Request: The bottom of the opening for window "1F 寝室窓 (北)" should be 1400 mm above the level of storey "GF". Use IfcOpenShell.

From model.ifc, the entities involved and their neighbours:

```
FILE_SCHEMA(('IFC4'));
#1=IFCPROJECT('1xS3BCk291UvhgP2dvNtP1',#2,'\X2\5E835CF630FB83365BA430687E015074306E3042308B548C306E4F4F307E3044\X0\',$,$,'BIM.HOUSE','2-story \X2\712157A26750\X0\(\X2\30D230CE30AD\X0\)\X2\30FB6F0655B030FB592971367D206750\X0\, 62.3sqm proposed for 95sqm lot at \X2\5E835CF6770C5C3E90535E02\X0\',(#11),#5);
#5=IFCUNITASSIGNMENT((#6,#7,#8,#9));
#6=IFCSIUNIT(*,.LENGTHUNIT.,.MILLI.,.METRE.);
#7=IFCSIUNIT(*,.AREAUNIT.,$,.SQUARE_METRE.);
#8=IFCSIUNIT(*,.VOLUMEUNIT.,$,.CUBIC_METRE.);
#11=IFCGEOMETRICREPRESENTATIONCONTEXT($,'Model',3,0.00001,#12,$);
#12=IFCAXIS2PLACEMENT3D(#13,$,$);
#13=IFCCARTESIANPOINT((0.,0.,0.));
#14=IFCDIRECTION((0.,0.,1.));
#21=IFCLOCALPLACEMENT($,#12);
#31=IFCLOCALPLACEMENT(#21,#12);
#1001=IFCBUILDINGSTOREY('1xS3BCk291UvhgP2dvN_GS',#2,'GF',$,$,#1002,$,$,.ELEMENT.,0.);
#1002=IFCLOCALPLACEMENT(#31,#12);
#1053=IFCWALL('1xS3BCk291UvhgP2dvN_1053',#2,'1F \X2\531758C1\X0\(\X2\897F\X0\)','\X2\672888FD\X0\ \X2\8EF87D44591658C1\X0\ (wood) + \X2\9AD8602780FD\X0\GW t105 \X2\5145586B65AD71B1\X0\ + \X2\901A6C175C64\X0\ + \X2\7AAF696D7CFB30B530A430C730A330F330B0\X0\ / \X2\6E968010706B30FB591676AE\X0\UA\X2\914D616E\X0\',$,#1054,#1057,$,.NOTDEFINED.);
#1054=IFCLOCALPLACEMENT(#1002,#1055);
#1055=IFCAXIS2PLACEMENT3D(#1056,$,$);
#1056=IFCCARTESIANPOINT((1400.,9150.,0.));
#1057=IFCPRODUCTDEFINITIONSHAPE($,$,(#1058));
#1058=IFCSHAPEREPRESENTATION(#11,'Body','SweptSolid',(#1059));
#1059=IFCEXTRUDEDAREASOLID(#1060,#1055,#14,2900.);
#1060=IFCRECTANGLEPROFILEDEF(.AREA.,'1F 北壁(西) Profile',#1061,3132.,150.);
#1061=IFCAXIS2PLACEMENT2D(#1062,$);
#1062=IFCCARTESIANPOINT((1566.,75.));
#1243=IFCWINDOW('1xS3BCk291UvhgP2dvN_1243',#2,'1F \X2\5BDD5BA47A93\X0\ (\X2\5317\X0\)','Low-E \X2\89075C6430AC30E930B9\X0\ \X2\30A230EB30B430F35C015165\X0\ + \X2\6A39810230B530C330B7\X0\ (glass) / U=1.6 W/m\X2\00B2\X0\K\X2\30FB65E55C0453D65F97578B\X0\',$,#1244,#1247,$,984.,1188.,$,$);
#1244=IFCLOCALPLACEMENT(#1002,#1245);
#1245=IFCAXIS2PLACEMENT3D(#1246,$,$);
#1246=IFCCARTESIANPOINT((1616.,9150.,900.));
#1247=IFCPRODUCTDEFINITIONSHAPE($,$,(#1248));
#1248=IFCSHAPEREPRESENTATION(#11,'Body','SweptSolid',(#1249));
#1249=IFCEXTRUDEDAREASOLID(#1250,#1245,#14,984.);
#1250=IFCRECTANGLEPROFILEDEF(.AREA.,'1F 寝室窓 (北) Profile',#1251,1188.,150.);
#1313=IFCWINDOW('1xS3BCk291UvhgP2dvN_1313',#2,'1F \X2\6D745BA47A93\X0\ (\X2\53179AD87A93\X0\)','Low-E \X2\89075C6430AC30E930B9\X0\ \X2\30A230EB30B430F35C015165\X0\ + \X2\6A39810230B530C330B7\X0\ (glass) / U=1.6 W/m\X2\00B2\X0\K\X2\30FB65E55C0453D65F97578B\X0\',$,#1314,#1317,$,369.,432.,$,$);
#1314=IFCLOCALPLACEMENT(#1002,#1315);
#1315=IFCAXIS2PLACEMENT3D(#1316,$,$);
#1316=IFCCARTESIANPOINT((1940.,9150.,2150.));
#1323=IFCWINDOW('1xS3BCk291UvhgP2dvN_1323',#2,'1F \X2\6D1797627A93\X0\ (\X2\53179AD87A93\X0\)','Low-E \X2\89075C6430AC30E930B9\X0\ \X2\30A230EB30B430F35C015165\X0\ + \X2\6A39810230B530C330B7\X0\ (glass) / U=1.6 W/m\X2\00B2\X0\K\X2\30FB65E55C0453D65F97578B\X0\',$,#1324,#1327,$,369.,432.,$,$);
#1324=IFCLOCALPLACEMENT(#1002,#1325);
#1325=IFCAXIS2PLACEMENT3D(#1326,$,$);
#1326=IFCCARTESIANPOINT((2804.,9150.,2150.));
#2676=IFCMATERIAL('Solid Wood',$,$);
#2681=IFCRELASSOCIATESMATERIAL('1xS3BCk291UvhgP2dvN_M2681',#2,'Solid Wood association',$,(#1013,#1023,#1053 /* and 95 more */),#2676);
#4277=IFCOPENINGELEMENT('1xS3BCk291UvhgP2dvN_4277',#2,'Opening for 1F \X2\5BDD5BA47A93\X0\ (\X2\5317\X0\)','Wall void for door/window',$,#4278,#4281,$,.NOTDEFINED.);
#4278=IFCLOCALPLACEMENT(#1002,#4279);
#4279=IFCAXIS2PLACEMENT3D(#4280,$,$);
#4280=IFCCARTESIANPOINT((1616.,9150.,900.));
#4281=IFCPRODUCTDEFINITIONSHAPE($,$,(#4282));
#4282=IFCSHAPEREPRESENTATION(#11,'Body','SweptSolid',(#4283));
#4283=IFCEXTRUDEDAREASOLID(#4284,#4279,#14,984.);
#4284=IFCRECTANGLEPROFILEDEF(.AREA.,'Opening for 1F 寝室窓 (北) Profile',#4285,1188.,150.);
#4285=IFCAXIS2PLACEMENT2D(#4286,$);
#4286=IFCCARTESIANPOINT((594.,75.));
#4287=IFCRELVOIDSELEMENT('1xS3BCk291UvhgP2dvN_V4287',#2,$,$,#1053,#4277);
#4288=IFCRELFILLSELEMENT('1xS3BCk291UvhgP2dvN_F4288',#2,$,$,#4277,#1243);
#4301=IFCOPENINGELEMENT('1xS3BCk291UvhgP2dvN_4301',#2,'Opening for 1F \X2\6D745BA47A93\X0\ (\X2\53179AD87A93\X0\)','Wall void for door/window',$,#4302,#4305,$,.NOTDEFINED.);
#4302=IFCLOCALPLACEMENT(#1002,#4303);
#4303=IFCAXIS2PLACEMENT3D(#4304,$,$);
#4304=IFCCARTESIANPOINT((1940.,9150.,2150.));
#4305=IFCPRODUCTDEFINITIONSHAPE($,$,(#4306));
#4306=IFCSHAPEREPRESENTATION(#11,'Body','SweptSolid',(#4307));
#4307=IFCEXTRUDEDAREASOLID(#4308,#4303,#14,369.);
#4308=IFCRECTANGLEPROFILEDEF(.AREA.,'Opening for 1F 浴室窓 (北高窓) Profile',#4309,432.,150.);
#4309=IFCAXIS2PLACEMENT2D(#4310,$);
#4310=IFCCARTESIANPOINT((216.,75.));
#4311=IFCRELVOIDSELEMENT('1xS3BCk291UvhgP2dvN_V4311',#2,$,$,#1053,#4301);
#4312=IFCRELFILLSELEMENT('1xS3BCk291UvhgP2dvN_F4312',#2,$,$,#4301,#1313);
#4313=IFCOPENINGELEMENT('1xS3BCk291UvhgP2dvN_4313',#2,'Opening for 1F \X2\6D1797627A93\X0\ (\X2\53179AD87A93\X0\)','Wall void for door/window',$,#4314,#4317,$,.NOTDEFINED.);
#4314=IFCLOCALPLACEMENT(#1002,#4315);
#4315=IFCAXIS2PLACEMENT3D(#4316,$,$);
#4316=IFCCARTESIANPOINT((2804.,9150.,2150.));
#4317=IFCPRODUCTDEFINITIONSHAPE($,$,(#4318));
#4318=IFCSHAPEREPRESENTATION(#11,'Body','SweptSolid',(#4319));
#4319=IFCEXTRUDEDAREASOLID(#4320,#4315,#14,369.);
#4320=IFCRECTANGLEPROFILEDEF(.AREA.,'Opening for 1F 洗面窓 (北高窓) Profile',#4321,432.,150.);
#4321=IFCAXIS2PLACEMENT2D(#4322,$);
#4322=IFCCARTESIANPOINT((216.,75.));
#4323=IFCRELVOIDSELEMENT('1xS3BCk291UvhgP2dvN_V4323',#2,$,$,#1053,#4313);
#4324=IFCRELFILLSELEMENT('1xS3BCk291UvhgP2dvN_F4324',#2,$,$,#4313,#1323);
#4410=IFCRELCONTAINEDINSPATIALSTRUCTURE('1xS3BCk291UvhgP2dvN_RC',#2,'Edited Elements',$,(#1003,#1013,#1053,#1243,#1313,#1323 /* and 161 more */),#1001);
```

```python
import numpy as np
import ifcopenshell
import ifcopenshell.api.geometry
import ifcopenshell.geom
import ifcopenshell.util.element
import ifcopenshell.util.placement
import ifcopenshell.util.shape
import ifcopenshell.util.unit

model = ifcopenshell.open("model.ifc")
unit_scale = ifcopenshell.util.unit.calculate_unit_scale(model)

window = model.by_id(1243)
opening = window.FillsVoids[0].RelatingOpeningElement
storey = ifcopenshell.util.element.get_container(window, ifc_class="IfcBuildingStorey")
level = ifcopenshell.util.placement.get_local_placement(storey.ObjectPlacement)[2, 3]

# The opening's origin need not be at the sill, so measure its lowest point.
shape = ifcopenshell.geom.create_shape(ifcopenshell.geom.settings(), opening)
bottom = ifcopenshell.util.shape.get_shape_bottom_elevation(shape, shape.geometry) / unit_scale
dz = level + 1400.0 - bottom

shift = np.array([0.0, 0.0, dz])
# The window is not placed relative to its opening, so move both.
for product in (opening, window):
    matrix = ifcopenshell.util.placement.get_local_placement(product.ObjectPlacement)
    matrix[:3, 3] += shift
    ifcopenshell.api.geometry.edit_object_placement(model, product=product, matrix=matrix, is_si=False)

print(f"moved by {dz * unit_scale:+.3f} m")

model.write("model_edited.ifc")
```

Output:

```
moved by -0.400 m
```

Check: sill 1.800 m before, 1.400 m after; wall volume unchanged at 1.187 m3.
